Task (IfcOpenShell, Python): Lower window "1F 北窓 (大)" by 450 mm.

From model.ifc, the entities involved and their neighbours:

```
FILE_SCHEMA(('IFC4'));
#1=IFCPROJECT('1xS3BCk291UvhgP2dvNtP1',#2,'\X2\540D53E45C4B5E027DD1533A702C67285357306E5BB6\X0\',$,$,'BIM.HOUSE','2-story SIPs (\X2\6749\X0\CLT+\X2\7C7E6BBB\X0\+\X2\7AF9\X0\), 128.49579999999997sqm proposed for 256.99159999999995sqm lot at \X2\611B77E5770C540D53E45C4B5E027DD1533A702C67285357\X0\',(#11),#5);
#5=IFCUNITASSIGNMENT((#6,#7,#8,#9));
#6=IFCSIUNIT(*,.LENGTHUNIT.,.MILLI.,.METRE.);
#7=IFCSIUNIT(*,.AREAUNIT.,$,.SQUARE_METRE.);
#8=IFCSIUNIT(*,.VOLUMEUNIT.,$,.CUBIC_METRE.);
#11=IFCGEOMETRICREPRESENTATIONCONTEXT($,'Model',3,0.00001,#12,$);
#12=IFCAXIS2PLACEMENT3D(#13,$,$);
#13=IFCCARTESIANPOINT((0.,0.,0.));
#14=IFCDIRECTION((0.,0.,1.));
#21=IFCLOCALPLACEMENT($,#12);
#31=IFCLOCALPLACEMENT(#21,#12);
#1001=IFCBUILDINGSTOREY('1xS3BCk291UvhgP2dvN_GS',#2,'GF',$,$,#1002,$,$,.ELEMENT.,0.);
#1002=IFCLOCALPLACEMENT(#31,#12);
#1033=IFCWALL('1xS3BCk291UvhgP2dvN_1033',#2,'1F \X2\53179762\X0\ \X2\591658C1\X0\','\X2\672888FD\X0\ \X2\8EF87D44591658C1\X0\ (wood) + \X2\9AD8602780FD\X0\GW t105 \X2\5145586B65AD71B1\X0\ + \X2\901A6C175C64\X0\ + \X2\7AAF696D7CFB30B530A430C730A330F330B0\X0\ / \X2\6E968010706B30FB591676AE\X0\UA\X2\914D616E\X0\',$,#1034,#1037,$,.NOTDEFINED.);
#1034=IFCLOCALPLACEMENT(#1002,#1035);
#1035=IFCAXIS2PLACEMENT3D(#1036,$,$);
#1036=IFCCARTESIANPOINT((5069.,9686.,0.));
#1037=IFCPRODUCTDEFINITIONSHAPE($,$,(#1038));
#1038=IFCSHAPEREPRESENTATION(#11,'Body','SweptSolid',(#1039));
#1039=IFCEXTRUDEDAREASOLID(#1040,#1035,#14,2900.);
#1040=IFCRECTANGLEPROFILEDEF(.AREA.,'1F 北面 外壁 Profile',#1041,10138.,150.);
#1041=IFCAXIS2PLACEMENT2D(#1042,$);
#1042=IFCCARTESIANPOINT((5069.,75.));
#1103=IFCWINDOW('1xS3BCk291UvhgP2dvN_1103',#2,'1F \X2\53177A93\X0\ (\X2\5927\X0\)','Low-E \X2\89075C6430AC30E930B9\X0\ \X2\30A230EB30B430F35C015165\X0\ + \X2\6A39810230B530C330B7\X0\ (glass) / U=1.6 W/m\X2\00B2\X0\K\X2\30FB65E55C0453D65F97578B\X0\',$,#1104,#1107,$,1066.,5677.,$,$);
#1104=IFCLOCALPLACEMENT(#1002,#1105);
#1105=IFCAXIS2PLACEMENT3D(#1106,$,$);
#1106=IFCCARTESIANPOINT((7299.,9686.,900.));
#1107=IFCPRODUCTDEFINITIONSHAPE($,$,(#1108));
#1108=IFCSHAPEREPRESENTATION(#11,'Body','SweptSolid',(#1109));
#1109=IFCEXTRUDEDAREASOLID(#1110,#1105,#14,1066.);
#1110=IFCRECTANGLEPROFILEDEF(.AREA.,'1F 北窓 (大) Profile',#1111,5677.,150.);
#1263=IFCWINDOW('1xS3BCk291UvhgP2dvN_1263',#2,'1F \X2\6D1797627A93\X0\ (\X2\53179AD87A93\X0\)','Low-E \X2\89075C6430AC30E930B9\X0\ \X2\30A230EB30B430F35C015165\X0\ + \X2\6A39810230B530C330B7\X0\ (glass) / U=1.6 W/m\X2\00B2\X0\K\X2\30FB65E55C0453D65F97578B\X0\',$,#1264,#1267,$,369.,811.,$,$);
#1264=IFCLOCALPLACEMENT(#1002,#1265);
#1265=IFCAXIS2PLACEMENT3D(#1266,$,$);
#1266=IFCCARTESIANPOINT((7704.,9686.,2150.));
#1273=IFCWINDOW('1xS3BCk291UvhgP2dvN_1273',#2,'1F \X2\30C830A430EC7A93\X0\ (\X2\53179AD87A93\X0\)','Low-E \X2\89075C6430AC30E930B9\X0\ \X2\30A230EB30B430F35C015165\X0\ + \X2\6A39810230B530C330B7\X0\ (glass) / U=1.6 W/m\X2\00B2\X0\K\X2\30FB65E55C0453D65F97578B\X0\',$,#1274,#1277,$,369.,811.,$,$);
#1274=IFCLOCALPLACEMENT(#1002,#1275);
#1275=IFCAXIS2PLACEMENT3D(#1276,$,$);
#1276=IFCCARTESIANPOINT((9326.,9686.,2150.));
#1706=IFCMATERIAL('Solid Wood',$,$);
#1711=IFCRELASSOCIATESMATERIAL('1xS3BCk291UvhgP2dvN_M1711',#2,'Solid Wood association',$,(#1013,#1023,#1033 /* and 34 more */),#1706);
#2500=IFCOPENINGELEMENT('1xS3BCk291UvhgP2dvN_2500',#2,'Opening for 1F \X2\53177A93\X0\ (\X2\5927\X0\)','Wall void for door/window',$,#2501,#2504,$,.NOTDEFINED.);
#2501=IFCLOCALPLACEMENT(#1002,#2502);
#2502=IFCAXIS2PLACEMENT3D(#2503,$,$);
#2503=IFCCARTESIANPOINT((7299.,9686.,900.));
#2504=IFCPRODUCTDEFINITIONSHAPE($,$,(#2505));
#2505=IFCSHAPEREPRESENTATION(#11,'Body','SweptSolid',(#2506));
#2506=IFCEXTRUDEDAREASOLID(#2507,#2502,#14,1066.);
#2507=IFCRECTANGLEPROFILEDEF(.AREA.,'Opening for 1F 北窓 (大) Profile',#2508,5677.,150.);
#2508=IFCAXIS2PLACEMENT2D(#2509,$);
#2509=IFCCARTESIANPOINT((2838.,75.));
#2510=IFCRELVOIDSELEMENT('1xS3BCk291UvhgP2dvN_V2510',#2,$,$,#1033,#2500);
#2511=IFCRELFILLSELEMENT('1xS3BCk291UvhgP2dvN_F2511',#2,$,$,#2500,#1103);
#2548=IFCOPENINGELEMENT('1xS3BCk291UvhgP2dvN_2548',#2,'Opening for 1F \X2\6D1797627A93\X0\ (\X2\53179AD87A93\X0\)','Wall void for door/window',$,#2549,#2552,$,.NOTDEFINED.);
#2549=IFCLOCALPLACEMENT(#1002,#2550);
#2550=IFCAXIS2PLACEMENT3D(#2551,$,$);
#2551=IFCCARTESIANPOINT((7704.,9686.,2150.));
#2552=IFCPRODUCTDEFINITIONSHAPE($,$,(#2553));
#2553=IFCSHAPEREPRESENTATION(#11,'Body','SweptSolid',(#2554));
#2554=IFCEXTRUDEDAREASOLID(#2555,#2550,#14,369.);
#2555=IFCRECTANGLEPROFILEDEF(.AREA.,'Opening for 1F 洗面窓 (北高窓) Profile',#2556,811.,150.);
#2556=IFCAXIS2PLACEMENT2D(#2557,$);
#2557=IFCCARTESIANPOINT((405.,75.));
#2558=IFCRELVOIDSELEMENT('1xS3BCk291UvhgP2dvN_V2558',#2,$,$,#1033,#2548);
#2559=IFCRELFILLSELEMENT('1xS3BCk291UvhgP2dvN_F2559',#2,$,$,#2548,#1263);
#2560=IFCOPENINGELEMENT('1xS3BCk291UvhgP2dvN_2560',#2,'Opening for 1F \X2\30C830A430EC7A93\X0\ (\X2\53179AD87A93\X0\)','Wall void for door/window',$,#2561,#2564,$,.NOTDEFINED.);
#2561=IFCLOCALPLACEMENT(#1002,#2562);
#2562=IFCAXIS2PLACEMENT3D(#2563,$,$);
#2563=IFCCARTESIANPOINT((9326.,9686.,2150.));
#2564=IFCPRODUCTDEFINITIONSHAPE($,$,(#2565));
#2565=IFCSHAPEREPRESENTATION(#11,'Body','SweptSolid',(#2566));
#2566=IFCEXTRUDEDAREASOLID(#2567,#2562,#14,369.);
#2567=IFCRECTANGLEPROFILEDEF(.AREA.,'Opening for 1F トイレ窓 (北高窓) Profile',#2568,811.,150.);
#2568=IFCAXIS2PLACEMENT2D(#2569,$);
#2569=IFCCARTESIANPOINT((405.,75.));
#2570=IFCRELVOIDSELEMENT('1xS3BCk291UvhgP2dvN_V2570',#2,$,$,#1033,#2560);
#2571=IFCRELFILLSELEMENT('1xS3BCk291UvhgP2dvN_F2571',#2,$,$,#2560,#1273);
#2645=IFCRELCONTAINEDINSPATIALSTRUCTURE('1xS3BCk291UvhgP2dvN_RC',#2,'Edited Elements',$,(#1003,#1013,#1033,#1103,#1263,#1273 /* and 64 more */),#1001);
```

```python
import numpy as np
import ifcopenshell
import ifcopenshell.api.geometry
import ifcopenshell.util.placement
import ifcopenshell.util.unit

model = ifcopenshell.open("model.ifc")
unit_scale = ifcopenshell.util.unit.calculate_unit_scale(model)

window = model.by_id(1103)
opening = window.FillsVoids[0].RelatingOpeningElement
dz = -450.0

shift = np.array([0.0, 0.0, dz])
# The window is not placed relative to its opening, so move both.
for product in (opening, window):
    matrix = ifcopenshell.util.placement.get_local_placement(product.ObjectPlacement)
    matrix[:3, 3] += shift
    ifcopenshell.api.geometry.edit_object_placement(model, product=product, matrix=matrix, is_si=False)

print(f"moved by {dz * unit_scale:+.3f} m")

model.write("model-out.ifc")
```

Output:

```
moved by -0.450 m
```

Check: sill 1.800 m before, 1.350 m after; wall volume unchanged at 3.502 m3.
